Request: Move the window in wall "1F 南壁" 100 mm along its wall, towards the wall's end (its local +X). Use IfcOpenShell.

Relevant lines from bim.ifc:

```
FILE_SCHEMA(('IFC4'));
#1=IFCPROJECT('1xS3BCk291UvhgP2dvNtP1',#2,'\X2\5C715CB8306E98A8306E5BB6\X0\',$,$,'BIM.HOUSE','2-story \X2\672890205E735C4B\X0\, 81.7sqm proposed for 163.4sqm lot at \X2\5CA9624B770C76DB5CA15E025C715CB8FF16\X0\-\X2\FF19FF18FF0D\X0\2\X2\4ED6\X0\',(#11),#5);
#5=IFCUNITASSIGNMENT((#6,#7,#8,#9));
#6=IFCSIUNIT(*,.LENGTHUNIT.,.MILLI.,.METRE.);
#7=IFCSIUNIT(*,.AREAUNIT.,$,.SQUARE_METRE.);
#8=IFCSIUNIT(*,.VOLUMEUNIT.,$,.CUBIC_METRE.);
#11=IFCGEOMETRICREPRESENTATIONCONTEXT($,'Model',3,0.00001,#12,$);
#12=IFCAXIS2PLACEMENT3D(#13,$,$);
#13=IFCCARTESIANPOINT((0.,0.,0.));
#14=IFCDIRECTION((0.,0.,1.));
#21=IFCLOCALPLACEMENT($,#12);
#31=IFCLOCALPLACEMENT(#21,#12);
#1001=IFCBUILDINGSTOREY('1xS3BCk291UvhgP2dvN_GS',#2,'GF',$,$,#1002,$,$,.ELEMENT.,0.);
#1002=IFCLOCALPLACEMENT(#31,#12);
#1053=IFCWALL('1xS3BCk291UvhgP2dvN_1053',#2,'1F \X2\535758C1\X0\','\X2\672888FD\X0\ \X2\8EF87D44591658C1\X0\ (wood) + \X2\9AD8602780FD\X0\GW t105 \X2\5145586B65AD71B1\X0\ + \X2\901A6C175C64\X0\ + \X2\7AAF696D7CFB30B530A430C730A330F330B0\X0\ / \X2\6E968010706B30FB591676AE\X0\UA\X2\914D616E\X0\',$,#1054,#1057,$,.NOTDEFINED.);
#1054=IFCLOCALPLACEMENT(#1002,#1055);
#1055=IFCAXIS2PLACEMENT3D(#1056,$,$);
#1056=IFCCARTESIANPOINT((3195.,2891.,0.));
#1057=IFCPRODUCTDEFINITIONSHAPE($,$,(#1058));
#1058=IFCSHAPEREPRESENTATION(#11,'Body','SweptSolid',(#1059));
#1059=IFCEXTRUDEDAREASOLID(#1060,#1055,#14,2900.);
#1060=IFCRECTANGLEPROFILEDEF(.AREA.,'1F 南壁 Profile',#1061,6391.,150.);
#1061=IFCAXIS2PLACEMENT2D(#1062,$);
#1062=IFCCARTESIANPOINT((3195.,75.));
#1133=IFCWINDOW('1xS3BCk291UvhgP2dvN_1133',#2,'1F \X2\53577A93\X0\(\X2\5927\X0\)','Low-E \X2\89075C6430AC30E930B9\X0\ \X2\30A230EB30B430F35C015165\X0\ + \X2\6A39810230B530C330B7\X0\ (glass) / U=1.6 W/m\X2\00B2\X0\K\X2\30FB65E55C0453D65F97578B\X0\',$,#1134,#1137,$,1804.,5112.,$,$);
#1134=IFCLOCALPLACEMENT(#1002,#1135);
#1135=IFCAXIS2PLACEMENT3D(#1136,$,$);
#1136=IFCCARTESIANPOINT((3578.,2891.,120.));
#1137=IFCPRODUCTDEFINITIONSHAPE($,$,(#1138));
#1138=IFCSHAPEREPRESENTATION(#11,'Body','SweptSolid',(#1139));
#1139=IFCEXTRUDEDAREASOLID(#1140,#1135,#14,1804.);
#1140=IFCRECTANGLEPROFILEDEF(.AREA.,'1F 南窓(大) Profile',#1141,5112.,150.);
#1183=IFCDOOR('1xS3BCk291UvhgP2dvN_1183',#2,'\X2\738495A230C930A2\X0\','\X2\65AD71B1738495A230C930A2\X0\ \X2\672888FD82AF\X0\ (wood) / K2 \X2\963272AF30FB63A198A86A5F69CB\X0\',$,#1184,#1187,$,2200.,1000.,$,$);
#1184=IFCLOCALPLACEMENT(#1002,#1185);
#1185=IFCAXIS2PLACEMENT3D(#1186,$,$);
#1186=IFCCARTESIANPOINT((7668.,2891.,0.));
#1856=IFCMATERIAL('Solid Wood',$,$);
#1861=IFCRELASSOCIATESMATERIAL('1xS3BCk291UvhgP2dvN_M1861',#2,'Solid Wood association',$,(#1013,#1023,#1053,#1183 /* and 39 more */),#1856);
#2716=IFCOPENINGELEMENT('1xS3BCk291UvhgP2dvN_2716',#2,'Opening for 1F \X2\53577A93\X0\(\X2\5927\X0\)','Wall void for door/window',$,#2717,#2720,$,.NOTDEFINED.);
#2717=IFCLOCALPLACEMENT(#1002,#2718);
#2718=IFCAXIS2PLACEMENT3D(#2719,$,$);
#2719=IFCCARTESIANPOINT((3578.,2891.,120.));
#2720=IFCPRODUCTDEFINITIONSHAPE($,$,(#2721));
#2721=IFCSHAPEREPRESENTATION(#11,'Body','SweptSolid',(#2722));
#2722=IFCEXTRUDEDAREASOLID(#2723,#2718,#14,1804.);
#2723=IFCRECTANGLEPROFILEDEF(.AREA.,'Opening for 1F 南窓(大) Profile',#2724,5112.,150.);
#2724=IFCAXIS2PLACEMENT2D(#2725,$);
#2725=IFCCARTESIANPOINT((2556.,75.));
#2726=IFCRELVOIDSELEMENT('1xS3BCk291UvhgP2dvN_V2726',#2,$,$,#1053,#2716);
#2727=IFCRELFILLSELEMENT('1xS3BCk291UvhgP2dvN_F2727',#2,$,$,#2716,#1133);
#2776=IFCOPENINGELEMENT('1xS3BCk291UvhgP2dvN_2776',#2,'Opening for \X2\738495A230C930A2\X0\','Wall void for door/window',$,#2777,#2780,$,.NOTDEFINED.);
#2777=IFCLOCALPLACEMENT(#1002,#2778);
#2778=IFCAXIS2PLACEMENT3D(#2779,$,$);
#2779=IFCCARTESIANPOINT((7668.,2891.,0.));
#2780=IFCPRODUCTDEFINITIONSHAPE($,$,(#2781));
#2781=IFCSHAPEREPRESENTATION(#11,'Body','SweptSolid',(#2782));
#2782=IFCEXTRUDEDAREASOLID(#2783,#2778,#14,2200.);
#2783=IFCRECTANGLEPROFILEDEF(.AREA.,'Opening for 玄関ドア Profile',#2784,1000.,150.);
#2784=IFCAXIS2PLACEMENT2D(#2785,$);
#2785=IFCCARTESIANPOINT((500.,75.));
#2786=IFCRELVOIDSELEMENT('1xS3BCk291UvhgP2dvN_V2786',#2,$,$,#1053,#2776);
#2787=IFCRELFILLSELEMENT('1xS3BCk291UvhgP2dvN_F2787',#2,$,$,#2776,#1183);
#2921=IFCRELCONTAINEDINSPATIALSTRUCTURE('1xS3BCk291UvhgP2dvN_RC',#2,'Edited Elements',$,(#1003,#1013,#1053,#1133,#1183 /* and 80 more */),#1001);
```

```python
import ifcopenshell
import ifcopenshell.api.geometry
import ifcopenshell.util.placement

model = ifcopenshell.open("bim.ifc")

window = model.by_guid("1xS3BCk291UvhgP2dvN_1133")
opening = window.FillsVoids[0].RelatingOpeningElement
wall = opening.VoidsElements[0].RelatingBuildingElement

wall_matrix = ifcopenshell.util.placement.get_local_placement(wall.ObjectPlacement)
shift = wall_matrix[:3, 0] * 100.0
before = ifcopenshell.util.placement.get_local_placement(window.ObjectPlacement)[:3, 3].copy()

# The window is not placed relative to its opening, so move both.
for product in (opening, window):
    matrix = ifcopenshell.util.placement.get_local_placement(product.ObjectPlacement)
    matrix[:3, 3] += shift
    ifcopenshell.api.geometry.edit_object_placement(model, product=product, matrix=matrix, is_si=False)

after = ifcopenshell.util.placement.get_local_placement(window.ObjectPlacement)[:3, 3]
print("window moved by", (after - before).round(3) + 0.0)

model.write("bim_updated.ifc")
```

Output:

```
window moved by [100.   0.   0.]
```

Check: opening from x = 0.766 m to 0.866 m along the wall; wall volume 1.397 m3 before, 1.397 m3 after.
